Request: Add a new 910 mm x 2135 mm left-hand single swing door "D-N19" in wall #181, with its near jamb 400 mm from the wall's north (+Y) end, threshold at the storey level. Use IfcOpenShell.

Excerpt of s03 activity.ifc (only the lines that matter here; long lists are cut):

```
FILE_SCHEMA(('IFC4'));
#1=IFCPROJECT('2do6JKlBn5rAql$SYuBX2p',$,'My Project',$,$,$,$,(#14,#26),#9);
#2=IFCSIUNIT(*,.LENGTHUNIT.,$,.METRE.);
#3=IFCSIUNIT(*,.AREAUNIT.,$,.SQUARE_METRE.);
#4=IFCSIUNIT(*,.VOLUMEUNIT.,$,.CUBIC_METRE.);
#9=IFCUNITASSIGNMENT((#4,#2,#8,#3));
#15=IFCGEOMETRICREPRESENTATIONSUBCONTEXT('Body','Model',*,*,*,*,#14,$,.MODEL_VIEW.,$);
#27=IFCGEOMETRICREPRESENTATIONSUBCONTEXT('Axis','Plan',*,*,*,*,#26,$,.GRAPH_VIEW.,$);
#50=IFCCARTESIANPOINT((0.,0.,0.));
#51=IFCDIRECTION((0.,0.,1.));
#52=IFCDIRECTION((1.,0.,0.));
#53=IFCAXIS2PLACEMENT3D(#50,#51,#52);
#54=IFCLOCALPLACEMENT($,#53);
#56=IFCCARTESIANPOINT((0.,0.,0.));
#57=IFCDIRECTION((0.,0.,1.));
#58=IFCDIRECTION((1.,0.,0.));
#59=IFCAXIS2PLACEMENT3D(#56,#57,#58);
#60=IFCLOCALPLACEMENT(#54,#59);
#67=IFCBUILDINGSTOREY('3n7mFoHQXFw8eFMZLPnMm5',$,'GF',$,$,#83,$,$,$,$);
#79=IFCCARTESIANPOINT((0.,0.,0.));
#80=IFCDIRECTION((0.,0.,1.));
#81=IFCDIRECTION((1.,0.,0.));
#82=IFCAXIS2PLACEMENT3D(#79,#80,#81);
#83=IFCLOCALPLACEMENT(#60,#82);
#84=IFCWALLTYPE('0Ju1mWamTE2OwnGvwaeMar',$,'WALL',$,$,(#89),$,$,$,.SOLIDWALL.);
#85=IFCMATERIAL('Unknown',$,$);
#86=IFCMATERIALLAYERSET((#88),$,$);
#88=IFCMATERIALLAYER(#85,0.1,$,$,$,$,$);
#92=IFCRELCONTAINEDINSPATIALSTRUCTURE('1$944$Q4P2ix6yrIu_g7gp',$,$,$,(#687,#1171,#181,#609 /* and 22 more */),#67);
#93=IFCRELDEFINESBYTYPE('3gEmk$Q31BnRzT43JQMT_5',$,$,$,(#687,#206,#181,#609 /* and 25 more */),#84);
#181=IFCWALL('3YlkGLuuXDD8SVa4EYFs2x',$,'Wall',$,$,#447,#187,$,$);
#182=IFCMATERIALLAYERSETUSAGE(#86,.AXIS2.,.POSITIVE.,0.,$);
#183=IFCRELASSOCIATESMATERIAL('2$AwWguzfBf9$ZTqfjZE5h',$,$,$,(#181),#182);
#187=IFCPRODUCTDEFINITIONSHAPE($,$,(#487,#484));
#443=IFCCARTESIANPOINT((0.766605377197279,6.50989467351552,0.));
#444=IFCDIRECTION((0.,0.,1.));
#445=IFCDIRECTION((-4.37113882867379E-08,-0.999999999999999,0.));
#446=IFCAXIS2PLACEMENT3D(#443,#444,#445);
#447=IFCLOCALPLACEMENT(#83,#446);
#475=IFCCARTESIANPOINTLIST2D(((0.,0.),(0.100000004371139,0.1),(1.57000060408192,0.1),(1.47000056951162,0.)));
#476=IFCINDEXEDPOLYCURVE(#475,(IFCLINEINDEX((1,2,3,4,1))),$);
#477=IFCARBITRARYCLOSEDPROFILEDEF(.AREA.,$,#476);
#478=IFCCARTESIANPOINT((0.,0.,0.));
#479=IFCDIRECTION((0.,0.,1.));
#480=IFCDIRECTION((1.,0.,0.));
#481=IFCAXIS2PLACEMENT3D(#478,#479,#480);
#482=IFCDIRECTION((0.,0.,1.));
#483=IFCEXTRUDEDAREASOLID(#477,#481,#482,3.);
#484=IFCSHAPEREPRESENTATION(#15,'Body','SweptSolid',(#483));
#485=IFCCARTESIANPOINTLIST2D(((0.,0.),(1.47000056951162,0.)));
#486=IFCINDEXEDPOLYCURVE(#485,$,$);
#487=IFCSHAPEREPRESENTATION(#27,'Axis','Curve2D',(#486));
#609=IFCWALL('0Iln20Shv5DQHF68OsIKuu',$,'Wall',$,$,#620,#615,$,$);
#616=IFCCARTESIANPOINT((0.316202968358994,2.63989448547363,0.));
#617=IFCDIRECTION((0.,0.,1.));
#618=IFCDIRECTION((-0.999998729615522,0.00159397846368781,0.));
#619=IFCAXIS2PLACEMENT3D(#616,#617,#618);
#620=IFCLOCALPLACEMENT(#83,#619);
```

```python
import numpy as np
import ifcopenshell
import ifcopenshell.api.feature
import ifcopenshell.api.geometry
import ifcopenshell.api.root
import ifcopenshell.api.spatial
import ifcopenshell.geom
import ifcopenshell.util.element
import ifcopenshell.util.placement
import ifcopenshell.util.representation
import ifcopenshell.util.shape
import ifcopenshell.util.unit

model = ifcopenshell.open("s03 activity.ifc")
unit_scale = ifcopenshell.util.unit.calculate_unit_scale(model)
settings = ifcopenshell.geom.settings()


def volume(element):
    """Net volume in cubic metres, openings subtracted."""
    shape = ifcopenshell.geom.create_shape(settings, element)
    return ifcopenshell.util.shape.get_volume(shape.geometry)


wall = model.by_guid("3YlkGLuuXDD8SVa4EYFs2x")
storey = ifcopenshell.util.element.get_container(wall, ifc_class="IfcBuildingStorey")
context = ifcopenshell.util.representation.get_context(model, "Model", "Body", "MODEL_VIEW")
before = volume(wall)

width, height, from_end, sill = 0.91, 2.135, 0.4, 0.0  # metres

# The wall runs along its own X axis, and the end named is its -X end.
wall_shape = ifcopenshell.geom.create_shape(settings, wall)
x, y, z = ifcopenshell.util.shape.get_vertices(wall_shape.geometry).T
start = x.min() + from_end
face, thickness = float(y.min()), float(y.max() - y.min())
wall_matrix = ifcopenshell.util.placement.get_local_placement(wall.ObjectPlacement)
level = ifcopenshell.util.placement.get_local_placement(storey.ObjectPlacement)[2, 3]


def in_wall(x, y):
    """Placement at x, y metres in the wall's axes, at sill height."""
    matrix = wall_matrix.copy()
    matrix[:, 3] = wall_matrix @ np.array([x / unit_scale, y / unit_scale, 0.0, 1.0])
    matrix[2, 3] = level + sill / unit_scale
    return matrix


# Opening: a box that overshoots both wall faces by 50 mm.
opening = ifcopenshell.api.root.create_entity(model, ifc_class="IfcOpeningElement", predefined_type="OPENING")
box = ifcopenshell.api.geometry.add_wall_representation(
    model, context=context, length=width, height=height, thickness=thickness + 0.1
)
ifcopenshell.api.geometry.assign_representation(model, product=opening, representation=box)
ifcopenshell.api.geometry.edit_object_placement(model, product=opening, matrix=in_wall(start, face - 0.05), is_si=False)
ifcopenshell.api.feature.add_feature(model, feature=opening, element=wall)

door = ifcopenshell.api.root.create_entity(model, ifc_class="IfcDoor", name="D-N19", predefined_type="DOOR")
door.OverallWidth, door.OverallHeight = width / unit_scale, height / unit_scale
door.OperationType = "SINGLE_SWING_LEFT"
body = ifcopenshell.api.geometry.add_door_representation(
    model,
    context=context,
    overall_width=door.OverallWidth,
    overall_height=door.OverallHeight,
    operation_type="SINGLE_SWING_LEFT",
    lining_properties={"LiningDepth": thickness / unit_scale, "ThresholdDepth": thickness / unit_scale},
)
ifcopenshell.api.geometry.assign_representation(model, product=door, representation=body)
ifcopenshell.api.spatial.assign_container(model, products=[door], relating_structure=storey)
ifcopenshell.api.feature.add_filling(model, opening=opening, element=door)

# The lining spans the wall, so the door starts at the wall face.
ifcopenshell.api.geometry.edit_object_placement(model, product=door, matrix=in_wall(start, face), is_si=False)

after = volume(wall)

print(f"wall volume {before:.3f} -> {after:.3f} m3")

model.write("s03 activity_updated.ifc")
```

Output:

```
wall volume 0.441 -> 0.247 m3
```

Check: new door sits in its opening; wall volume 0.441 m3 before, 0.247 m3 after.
